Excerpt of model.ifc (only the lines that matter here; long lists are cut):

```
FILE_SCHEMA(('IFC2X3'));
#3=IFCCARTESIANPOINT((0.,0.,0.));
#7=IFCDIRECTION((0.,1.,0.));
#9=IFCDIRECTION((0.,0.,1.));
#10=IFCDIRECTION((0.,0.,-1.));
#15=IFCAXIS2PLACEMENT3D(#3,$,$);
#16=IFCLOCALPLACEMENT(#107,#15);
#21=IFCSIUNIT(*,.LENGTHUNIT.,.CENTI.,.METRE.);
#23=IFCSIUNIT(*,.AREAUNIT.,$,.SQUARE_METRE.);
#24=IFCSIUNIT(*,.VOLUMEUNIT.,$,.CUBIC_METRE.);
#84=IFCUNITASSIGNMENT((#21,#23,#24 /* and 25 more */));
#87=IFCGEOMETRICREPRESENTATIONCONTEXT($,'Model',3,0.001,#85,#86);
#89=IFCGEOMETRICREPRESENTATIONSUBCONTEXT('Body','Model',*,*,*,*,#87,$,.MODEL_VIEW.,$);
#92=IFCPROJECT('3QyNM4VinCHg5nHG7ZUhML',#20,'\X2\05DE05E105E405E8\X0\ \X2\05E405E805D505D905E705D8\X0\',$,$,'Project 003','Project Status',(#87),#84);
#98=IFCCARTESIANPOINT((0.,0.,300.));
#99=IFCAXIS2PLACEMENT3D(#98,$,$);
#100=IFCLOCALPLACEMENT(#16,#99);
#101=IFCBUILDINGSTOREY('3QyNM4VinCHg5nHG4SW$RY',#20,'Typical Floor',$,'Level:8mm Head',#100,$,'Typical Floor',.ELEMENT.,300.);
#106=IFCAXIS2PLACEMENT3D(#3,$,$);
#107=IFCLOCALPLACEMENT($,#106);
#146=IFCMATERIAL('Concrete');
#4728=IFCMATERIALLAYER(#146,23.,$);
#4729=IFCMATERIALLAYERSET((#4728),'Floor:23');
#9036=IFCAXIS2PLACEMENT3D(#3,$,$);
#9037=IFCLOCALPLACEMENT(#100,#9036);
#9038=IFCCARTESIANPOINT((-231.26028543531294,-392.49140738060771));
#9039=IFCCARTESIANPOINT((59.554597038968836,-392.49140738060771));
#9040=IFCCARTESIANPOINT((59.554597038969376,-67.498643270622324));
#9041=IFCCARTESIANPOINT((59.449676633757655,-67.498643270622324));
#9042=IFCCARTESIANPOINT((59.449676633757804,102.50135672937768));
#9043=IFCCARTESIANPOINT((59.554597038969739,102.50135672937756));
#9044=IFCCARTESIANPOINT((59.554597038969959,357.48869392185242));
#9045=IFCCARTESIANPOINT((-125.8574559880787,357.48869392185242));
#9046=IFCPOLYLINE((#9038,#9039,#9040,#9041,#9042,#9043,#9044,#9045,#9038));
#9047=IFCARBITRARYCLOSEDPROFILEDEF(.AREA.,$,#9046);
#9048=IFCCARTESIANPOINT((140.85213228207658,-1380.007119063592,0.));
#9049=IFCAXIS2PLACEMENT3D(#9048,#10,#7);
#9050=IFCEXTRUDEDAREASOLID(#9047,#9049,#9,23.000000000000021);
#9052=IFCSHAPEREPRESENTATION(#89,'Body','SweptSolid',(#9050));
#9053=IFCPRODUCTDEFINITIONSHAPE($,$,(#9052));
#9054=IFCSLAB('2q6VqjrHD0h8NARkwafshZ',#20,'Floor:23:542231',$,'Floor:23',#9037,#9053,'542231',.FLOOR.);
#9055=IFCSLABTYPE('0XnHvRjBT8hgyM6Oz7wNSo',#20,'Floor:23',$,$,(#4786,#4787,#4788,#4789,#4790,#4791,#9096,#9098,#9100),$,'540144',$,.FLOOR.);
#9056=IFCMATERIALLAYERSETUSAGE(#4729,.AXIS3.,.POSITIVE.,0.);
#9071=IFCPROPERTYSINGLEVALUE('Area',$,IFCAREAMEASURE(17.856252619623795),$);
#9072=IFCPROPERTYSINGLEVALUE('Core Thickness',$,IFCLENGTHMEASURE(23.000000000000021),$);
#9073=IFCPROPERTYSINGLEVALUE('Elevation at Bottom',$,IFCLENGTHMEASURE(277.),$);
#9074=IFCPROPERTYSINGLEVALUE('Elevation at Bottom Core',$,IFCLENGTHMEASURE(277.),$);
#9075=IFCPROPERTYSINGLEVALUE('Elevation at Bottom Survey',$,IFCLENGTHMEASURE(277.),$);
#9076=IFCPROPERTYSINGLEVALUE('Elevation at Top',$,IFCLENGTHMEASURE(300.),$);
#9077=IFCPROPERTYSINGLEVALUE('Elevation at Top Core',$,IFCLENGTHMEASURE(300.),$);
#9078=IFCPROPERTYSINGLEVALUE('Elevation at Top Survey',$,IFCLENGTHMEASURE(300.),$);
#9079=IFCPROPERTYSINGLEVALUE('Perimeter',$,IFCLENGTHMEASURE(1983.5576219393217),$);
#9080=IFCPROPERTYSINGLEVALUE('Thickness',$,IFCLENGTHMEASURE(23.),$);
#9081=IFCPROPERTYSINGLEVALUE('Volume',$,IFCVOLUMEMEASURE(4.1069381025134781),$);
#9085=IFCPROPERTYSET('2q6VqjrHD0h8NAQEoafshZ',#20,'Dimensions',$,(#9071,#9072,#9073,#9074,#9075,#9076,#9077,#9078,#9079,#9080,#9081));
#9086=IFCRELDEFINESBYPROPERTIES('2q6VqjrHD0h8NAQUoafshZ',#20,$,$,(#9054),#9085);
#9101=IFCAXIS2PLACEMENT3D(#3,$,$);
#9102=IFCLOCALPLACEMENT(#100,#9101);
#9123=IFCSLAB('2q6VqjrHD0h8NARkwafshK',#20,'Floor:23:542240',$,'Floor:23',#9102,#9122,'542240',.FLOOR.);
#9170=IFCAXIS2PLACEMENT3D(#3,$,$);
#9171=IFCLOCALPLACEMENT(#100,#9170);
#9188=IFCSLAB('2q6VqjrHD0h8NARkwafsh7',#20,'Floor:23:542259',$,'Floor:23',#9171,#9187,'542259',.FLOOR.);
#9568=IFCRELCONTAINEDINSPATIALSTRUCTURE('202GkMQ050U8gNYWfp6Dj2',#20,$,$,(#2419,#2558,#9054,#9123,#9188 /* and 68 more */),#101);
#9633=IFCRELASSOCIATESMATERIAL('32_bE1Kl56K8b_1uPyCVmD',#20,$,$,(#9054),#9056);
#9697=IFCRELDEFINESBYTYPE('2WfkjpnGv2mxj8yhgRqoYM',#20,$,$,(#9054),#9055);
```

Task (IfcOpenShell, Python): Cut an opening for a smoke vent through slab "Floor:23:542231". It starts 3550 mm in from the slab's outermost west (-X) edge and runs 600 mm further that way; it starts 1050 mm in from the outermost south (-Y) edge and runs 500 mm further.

```python
import numpy as np
import ifcopenshell
import ifcopenshell.api.feature
import ifcopenshell.api.geometry
import ifcopenshell.api.pset
import ifcopenshell.api.root
import ifcopenshell.geom
import ifcopenshell.util.element
import ifcopenshell.util.placement
import ifcopenshell.util.representation
import ifcopenshell.util.shape
import ifcopenshell.util.unit

model = ifcopenshell.open("model.ifc")
unit_scale = ifcopenshell.util.unit.calculate_unit_scale(model)
area_scale = ifcopenshell.util.unit.calculate_unit_scale(model, "AREAUNIT")
volume_scale = ifcopenshell.util.unit.calculate_unit_scale(model, "VOLUMEUNIT")
settings = ifcopenshell.geom.settings()


def volume(element):
    """Net volume in cubic metres, openings subtracted."""
    shape = ifcopenshell.geom.create_shape(settings, element)
    return ifcopenshell.util.shape.get_volume(shape.geometry)


slab = model.by_guid("2q6VqjrHD0h8NARkwafshZ")
before = volume(slab)

# Extent in the slab's own axes, in metres. The edges named are its -X and -Y sides.
slab_shape = ifcopenshell.geom.create_shape(settings, slab)
vertices = ifcopenshell.util.shape.get_vertices(slab_shape.geometry)
x_min, y_min, bottom = vertices.min(axis=0)
top = vertices[:, 2].max()

opening = ifcopenshell.api.root.create_entity(model, ifc_class="IfcOpeningElement", name="Smoke vent opening")
context = ifcopenshell.util.representation.get_context(model, "Model", "Body", "MODEL_VIEW")
width, depth = 0.6, 0.5
outline = [(0.0, 0.0), (width, 0.0), (width, depth), (0.0, depth), (0.0, 0.0)]
# Overshoot both faces by 50 mm so the cut is clean.
shape = ifcopenshell.api.geometry.add_slab_representation(
    model, context=context, depth=top - bottom + 0.1, polyline=outline
)
ifcopenshell.api.geometry.assign_representation(model, product=opening, representation=shape)

matrix = ifcopenshell.util.placement.get_local_placement(slab.ObjectPlacement)
matrix[:, 3] = matrix @ np.append(np.array([x_min + 3.55, y_min + 1.05, bottom - 0.05]) / unit_scale, 1.0)
ifcopenshell.api.geometry.edit_object_placement(model, product=opening, matrix=matrix, is_si=False)
ifcopenshell.api.feature.add_feature(model, feature=opening, element=slab)

after = volume(slab)

# Update the slab's stored quantities.
pset = model.by_id(ifcopenshell.util.element.get_pset(slab, "Dimensions", should_inherit=False)["id"])
ifcopenshell.api.pset.edit_pset(model, pset=pset, properties={
    "Area": model.create_entity("IfcAreaMeasure", after / (top - bottom) / area_scale),
    "Volume": model.create_entity("IfcVolumeMeasure", after / volume_scale),
})

print(f"slab volume {before:.3f} -> {after:.3f} m3")

model.write("model-out.ifc")
```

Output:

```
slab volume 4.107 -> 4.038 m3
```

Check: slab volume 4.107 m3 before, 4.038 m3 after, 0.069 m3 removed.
